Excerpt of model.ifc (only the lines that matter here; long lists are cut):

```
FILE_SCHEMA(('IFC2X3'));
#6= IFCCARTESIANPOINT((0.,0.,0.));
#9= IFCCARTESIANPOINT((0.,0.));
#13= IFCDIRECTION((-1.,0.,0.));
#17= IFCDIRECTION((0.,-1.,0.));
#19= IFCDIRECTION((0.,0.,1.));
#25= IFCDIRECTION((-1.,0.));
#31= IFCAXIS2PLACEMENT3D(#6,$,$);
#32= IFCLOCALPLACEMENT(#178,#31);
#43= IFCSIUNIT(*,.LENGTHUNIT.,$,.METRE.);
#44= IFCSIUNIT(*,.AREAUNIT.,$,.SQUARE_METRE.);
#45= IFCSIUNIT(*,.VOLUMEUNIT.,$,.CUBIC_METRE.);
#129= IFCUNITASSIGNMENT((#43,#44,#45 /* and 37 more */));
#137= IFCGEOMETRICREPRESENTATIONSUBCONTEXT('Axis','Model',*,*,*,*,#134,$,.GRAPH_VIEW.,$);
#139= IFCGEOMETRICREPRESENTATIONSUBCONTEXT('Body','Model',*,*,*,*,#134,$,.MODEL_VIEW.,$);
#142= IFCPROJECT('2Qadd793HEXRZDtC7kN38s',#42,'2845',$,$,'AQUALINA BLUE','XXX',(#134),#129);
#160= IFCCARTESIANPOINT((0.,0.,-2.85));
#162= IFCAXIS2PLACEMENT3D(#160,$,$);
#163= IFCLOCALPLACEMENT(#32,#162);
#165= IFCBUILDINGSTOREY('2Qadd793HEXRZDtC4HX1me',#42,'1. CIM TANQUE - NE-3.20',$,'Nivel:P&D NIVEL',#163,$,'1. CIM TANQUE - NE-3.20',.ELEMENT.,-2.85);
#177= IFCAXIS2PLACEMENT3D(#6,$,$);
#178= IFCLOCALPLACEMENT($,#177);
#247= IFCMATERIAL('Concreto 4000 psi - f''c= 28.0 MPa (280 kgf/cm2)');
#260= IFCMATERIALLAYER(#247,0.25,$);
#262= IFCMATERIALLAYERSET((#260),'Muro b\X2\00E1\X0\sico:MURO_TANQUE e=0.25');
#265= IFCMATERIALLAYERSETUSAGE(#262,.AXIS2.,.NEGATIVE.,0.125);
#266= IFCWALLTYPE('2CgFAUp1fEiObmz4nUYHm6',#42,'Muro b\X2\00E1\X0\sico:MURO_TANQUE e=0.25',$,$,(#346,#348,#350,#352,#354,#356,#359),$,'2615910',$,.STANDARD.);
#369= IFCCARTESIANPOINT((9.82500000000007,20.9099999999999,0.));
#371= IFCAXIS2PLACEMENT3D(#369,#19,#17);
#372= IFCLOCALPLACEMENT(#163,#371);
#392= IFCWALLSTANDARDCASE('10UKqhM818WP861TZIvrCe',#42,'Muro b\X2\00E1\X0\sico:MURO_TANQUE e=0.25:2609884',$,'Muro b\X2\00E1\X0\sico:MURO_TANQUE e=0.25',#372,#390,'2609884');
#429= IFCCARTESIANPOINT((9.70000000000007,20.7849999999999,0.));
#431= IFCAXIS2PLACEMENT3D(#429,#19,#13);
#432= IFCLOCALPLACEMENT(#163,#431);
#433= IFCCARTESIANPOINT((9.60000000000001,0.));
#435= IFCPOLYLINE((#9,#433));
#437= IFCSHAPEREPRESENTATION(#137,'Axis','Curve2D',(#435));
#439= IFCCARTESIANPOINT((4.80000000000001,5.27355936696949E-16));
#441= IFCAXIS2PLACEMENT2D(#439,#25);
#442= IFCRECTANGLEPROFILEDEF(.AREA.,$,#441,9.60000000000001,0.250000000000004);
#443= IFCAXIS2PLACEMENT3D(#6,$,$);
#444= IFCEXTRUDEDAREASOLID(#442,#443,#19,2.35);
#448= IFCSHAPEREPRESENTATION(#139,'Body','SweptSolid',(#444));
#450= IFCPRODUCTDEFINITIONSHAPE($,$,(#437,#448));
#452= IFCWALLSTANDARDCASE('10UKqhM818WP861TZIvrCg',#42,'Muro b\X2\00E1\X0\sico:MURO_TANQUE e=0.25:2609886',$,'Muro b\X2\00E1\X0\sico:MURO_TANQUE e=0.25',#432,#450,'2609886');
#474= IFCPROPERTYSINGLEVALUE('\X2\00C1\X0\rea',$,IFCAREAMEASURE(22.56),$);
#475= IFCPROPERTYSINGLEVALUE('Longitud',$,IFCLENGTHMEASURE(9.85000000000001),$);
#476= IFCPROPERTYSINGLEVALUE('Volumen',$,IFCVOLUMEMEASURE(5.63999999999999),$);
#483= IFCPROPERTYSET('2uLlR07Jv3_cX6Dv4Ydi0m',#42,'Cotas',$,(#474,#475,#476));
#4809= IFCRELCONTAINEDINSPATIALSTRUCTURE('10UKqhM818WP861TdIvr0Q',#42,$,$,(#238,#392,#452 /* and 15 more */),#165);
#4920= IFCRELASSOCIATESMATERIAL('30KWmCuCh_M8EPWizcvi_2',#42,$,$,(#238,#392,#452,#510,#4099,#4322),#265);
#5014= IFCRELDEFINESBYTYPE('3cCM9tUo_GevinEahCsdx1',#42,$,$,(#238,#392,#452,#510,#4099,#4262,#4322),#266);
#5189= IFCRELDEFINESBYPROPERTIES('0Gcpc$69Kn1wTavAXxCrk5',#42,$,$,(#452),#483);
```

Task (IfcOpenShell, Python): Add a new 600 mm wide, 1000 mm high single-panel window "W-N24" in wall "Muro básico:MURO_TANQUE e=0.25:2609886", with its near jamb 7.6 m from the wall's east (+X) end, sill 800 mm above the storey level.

```python
import numpy as np
import ifcopenshell
import ifcopenshell.api.feature
import ifcopenshell.api.geometry
import ifcopenshell.api.pset
import ifcopenshell.api.root
import ifcopenshell.api.spatial
import ifcopenshell.api.type
import ifcopenshell.geom
import ifcopenshell.util.element
import ifcopenshell.util.placement
import ifcopenshell.util.representation
import ifcopenshell.util.shape
import ifcopenshell.util.unit

model = ifcopenshell.open("model.ifc")
unit_scale = ifcopenshell.util.unit.calculate_unit_scale(model)
area_scale = ifcopenshell.util.unit.calculate_unit_scale(model, "AREAUNIT")
volume_scale = ifcopenshell.util.unit.calculate_unit_scale(model, "VOLUMEUNIT")
settings = ifcopenshell.geom.settings()


def volume(element):
    """Net volume in cubic metres, openings subtracted."""
    shape = ifcopenshell.geom.create_shape(settings, element)
    return ifcopenshell.util.shape.get_volume(shape.geometry)


wall = model.by_guid("10UKqhM818WP861TZIvrCg")
storey = ifcopenshell.util.element.get_container(wall, ifc_class="IfcBuildingStorey")
context = ifcopenshell.util.representation.get_context(model, "Model", "Body", "MODEL_VIEW")
before = volume(wall)

width, height, from_end, sill = 0.6, 1, 7.6, 0.8  # metres

# The wall runs along its own X axis, and the end named is its -X end.
wall_shape = ifcopenshell.geom.create_shape(settings, wall)
x, y, z = ifcopenshell.util.shape.get_vertices(wall_shape.geometry).T
start = x.min() + from_end
face, thickness = float(y.min()), float(y.max() - y.min())
wall_matrix = ifcopenshell.util.placement.get_local_placement(wall.ObjectPlacement)
level = ifcopenshell.util.placement.get_local_placement(storey.ObjectPlacement)[2, 3]


def in_wall(x, y):
    """Placement at x, y metres in the wall's axes, at sill height."""
    matrix = wall_matrix.copy()
    matrix[:, 3] = wall_matrix @ np.array([x / unit_scale, y / unit_scale, 0.0, 1.0])
    matrix[2, 3] = level + sill / unit_scale
    return matrix


# Opening: a box that overshoots both wall faces by 50 mm.
opening = ifcopenshell.api.root.create_entity(model, ifc_class="IfcOpeningElement")
box = ifcopenshell.api.geometry.add_wall_representation(
    model, context=context, length=width, height=height, thickness=thickness + 0.1
)
ifcopenshell.api.geometry.assign_representation(model, product=opening, representation=box)
ifcopenshell.api.geometry.edit_object_placement(model, product=opening, matrix=in_wall(start, face - 0.05), is_si=False)
ifcopenshell.api.feature.add_feature(model, feature=opening, element=wall)

window = ifcopenshell.api.root.create_entity(model, ifc_class="IfcWindow", name="W-N24")
window.OverallWidth, window.OverallHeight = width / unit_scale, height / unit_scale
body = ifcopenshell.api.geometry.add_window_representation(
    model,
    context=context,
    overall_width=window.OverallWidth,
    overall_height=window.OverallHeight,
    partition_type="SINGLE_PANEL",
)
ifcopenshell.api.geometry.assign_representation(model, product=window, representation=body)
ifcopenshell.api.spatial.assign_container(model, products=[window], relating_structure=storey)
fills = ifcopenshell.api.feature.add_filling(model, opening=opening, element=window)
fills.OwnerHistory = window.OwnerHistory  # required in IFC2X3

# IFC2X3 keeps the operation on the window style.
style = ifcopenshell.api.root.create_entity(model, ifc_class="IfcWindowStyle", name="W-N24")
style.OperationType, style.ConstructionType = "SINGLE_PANEL", "NOTDEFINED"
style.ParameterTakesPrecedence = style.Sizeable = False
ifcopenshell.api.type.assign_type(model, related_objects=[window], relating_type=style)

# Centre the window in the wall's thickness.
ifcopenshell.api.geometry.edit_object_placement(model, product=window, matrix=in_wall(start, face), is_si=False)
window_shape = ifcopenshell.geom.create_shape(settings, window)
depth = ifcopenshell.util.shape.get_vertices(window_shape.geometry)[:, 1]
offset = face + thickness / 2 - (depth.min() + depth.max()) / 2
ifcopenshell.api.geometry.edit_object_placement(model, product=window, matrix=in_wall(start, offset), is_si=False)

after = volume(wall)

# Update the wall's stored quantities.
pset = model.by_id(ifcopenshell.util.element.get_pset(wall, "Cotas", should_inherit=False)["id"])
ifcopenshell.api.pset.edit_pset(model, pset=pset, properties={
    "Área": model.create_entity("IfcAreaMeasure", after / thickness / area_scale),
    "Volumen": model.create_entity("IfcVolumeMeasure", after / volume_scale),
})

print(f"wall volume {before:.3f} -> {after:.3f} m3")

model.write("model-out.ifc")
```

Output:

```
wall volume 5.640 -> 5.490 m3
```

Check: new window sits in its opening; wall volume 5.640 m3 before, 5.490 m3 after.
